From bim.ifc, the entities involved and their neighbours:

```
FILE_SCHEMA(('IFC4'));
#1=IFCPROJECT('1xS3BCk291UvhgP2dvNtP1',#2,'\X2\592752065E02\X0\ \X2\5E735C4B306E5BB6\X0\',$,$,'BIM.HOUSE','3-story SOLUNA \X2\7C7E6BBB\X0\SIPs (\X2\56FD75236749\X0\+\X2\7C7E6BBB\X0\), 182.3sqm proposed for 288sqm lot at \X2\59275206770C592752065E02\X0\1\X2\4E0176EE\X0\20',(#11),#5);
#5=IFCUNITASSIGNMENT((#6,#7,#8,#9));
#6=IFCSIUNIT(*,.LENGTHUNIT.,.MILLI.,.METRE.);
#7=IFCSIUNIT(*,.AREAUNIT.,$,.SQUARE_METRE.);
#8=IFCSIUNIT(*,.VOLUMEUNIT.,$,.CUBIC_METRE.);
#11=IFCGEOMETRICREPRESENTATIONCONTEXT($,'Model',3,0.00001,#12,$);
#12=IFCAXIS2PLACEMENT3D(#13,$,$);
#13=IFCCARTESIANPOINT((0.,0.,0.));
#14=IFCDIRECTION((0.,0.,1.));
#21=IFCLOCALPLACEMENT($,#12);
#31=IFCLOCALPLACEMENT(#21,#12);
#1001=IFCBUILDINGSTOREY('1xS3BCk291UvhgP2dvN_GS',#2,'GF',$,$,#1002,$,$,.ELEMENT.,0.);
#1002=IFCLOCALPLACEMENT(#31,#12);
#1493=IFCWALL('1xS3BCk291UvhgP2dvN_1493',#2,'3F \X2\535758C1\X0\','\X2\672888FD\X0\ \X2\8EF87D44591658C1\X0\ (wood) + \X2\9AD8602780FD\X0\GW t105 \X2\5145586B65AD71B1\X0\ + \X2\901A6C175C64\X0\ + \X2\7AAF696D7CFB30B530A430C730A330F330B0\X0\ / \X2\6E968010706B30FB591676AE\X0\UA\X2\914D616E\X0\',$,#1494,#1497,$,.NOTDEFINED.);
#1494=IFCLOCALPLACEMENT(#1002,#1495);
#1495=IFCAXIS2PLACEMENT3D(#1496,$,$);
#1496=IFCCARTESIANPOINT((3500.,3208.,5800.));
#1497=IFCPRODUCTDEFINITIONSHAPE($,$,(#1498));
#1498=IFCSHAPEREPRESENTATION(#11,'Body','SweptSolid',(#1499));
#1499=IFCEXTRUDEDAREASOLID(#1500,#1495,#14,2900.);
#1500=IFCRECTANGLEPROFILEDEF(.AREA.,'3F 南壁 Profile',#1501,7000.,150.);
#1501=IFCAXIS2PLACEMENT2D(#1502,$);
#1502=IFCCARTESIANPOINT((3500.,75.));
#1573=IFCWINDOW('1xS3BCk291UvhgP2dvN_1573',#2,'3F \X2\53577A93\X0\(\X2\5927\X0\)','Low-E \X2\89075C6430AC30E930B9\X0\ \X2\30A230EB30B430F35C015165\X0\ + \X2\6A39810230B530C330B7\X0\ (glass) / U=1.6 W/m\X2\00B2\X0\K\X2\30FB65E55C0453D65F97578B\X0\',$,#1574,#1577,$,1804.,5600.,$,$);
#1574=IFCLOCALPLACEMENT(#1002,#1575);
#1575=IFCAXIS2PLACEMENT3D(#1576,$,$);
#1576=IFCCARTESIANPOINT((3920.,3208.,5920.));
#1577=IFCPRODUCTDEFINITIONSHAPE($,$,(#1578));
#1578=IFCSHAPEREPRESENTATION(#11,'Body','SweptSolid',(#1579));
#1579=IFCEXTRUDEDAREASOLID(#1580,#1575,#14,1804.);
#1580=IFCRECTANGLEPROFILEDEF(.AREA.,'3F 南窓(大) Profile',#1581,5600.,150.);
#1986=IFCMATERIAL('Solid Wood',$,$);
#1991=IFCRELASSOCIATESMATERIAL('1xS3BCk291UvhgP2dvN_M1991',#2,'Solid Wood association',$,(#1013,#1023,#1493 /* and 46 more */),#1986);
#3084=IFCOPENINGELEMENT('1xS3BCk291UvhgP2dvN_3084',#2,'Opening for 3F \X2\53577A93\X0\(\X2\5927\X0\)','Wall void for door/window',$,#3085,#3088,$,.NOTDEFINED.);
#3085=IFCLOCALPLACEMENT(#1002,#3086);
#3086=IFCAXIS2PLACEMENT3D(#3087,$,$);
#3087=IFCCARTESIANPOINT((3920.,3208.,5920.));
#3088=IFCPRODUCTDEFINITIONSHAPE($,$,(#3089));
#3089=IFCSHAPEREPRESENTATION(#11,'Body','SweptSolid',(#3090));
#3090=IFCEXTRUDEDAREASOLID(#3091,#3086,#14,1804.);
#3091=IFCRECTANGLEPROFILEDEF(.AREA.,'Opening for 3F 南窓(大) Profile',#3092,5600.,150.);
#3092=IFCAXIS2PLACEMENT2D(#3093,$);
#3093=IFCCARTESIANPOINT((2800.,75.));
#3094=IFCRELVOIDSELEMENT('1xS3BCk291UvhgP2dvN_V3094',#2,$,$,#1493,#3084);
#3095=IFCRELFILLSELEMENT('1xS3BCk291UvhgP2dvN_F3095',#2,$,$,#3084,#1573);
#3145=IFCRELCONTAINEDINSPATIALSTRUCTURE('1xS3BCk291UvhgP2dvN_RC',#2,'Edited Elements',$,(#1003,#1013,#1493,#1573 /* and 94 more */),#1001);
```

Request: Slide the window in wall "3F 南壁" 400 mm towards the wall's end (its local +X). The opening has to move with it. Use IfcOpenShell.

```python
import ifcopenshell
import ifcopenshell.api.geometry
import ifcopenshell.util.placement

model = ifcopenshell.open("bim.ifc")

window = model.by_id(1573)
opening = window.FillsVoids[0].RelatingOpeningElement
wall = opening.VoidsElements[0].RelatingBuildingElement

wall_matrix = ifcopenshell.util.placement.get_local_placement(wall.ObjectPlacement)
shift = wall_matrix[:3, 0] * 400.0
before = ifcopenshell.util.placement.get_local_placement(window.ObjectPlacement)[:3, 3].copy()

# The window is not placed relative to its opening, so move both.
for product in (opening, window):
    matrix = ifcopenshell.util.placement.get_local_placement(product.ObjectPlacement)
    matrix[:3, 3] += shift
    ifcopenshell.api.geometry.edit_object_placement(model, product=product, matrix=matrix, is_si=False)

after = ifcopenshell.util.placement.get_local_placement(window.ObjectPlacement)[:3, 3]
print("window moved by", (after - before).round(3) + 0.0)

model.write("bim_rev.ifc")
```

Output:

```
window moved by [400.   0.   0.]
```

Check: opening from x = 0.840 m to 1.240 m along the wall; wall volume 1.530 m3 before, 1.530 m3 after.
